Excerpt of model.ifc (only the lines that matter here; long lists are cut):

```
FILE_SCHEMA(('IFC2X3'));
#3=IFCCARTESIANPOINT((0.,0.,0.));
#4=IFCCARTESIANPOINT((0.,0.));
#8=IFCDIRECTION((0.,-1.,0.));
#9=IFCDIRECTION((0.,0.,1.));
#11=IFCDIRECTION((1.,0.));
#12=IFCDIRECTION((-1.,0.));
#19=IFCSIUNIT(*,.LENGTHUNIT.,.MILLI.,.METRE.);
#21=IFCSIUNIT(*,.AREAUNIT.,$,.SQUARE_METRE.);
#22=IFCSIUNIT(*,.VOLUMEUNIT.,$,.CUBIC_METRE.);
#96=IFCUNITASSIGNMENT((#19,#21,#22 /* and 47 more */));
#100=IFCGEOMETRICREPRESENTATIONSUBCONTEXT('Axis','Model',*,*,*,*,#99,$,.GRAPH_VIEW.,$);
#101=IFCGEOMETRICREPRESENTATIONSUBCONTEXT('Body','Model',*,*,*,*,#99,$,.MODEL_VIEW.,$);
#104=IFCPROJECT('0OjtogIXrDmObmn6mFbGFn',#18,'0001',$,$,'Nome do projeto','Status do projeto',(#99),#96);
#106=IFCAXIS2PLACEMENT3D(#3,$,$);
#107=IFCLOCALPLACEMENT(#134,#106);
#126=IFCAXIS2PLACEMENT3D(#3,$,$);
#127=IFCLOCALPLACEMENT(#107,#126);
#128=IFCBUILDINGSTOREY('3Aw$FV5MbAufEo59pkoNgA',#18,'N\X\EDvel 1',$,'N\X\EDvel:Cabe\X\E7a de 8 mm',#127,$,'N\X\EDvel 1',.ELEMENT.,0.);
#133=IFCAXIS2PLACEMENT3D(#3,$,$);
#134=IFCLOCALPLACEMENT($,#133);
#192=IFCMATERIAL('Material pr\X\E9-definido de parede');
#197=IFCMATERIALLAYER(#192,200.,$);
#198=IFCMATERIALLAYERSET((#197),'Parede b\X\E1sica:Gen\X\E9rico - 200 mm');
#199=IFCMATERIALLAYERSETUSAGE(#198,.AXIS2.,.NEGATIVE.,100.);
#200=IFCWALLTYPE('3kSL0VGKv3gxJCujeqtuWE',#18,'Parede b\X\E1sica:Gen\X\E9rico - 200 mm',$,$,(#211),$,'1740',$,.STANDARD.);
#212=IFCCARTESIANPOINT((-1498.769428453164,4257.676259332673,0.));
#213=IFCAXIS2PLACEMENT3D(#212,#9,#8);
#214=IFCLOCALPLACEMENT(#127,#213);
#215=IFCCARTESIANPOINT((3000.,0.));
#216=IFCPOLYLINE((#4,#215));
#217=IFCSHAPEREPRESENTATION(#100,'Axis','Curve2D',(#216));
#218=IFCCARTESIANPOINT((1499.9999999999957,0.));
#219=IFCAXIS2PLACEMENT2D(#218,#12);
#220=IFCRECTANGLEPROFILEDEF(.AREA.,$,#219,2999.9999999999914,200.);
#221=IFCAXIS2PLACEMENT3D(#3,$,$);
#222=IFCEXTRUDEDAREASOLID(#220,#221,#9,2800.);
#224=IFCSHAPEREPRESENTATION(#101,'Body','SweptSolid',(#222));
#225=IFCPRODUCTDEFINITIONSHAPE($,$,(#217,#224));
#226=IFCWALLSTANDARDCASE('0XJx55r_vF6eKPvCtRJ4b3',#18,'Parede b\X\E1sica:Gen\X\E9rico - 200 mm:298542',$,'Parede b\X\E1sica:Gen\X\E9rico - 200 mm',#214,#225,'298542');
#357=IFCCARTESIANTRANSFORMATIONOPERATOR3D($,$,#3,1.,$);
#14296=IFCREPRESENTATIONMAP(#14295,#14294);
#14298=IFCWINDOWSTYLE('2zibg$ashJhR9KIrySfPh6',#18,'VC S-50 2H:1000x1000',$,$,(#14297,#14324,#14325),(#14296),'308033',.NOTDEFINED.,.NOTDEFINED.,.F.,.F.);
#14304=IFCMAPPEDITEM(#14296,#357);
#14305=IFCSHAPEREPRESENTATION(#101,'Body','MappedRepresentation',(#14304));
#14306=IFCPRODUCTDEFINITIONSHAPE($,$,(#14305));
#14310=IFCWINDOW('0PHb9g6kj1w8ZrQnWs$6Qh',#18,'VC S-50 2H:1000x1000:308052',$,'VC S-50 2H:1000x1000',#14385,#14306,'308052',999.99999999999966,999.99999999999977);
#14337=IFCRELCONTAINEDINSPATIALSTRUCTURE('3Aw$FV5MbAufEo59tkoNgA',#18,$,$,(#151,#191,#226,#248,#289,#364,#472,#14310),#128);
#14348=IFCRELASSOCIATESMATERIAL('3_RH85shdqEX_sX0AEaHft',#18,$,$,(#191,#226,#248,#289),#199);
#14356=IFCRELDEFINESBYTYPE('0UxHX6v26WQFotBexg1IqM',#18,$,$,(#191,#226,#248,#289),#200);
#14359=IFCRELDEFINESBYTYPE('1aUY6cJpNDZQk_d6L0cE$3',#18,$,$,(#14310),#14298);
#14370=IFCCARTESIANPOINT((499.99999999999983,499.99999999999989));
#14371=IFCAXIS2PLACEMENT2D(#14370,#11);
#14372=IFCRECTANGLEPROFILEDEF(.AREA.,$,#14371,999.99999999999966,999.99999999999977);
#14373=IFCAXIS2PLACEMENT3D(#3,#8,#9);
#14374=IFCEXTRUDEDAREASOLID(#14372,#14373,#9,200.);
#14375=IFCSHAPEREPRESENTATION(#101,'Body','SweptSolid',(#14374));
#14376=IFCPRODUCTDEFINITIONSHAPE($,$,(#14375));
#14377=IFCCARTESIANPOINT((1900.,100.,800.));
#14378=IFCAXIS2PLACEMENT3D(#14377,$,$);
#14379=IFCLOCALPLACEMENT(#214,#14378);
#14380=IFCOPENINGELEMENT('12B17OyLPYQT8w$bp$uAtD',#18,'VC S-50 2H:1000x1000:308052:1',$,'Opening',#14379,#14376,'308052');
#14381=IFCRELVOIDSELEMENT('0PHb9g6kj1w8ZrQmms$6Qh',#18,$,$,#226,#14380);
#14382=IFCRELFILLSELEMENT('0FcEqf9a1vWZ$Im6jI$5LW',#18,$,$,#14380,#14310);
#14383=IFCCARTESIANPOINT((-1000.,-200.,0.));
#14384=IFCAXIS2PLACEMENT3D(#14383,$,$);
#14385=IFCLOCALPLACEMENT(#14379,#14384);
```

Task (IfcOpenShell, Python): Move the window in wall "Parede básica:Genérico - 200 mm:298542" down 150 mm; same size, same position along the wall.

```python
import numpy as np
import ifcopenshell
import ifcopenshell.api.geometry
import ifcopenshell.util.placement
import ifcopenshell.util.unit

model = ifcopenshell.open("model.ifc")
unit_scale = ifcopenshell.util.unit.calculate_unit_scale(model)

window = model.by_guid("0PHb9g6kj1w8ZrQnWs$6Qh")
opening = window.FillsVoids[0].RelatingOpeningElement
dz = -0.15 / unit_scale

shift = np.array([0.0, 0.0, dz])
# The window is placed relative to its opening, so it follows when the opening moves.
matrix = ifcopenshell.util.placement.get_local_placement(opening.ObjectPlacement)
matrix[:3, 3] += shift
ifcopenshell.api.geometry.edit_object_placement(
    model, product=opening, matrix=matrix, is_si=False, should_transform_children=True
)

print(f"moved by {dz * unit_scale:+.3f} m")

model.write("model-out.ifc")
```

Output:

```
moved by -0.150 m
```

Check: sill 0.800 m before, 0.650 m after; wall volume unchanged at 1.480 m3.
